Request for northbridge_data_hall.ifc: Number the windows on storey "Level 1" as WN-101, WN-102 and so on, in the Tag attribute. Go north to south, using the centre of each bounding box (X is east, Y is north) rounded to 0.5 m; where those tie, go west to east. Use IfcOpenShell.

First a look at what the model holds.

```python
import ifcopenshell
import ifcopenshell.util.element
import ifcopenshell.util.placement

model = ifcopenshell.open("northbridge_data_hall.ifc")
print(model.schema)
storey = next(s for s in model.by_type("IfcBuildingStorey") if s.Name == "Level 1")
windows = [e for e in ifcopenshell.util.element.get_decomposition(storey) if e.is_a("IfcWindow")]
for e in sorted(windows, key=lambda e: e.id()):
    origin = ifcopenshell.util.placement.get_local_placement(e.ObjectPlacement)[:3, 3]
    print(e.id(), e.Tag, e.Name, origin.round(2) + 0.0, sep=" | ")
```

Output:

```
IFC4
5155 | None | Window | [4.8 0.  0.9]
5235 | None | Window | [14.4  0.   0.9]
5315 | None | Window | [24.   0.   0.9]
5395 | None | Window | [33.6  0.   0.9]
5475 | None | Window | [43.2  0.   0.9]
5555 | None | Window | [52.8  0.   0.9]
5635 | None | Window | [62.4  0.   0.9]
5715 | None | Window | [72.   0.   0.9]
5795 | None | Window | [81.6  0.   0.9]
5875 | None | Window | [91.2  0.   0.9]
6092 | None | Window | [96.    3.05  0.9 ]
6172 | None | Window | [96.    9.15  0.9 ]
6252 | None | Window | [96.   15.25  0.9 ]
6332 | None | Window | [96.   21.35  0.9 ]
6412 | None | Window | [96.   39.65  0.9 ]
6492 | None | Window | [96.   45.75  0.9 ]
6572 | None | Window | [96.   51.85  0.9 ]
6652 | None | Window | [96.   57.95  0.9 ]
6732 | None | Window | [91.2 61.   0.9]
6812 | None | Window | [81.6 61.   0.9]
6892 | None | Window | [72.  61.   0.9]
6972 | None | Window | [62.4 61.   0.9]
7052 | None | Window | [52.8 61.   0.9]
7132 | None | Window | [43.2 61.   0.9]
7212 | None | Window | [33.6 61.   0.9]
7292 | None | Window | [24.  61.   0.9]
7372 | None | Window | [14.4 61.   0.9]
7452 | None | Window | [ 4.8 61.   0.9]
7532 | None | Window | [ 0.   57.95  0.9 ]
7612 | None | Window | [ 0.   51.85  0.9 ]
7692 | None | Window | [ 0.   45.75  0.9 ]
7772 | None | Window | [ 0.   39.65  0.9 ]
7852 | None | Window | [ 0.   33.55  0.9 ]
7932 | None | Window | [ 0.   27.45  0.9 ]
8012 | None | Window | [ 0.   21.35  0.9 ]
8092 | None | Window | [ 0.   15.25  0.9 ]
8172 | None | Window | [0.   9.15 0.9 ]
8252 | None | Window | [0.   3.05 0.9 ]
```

```python
import ifcopenshell
import ifcopenshell.geom
import ifcopenshell.util.element
import ifcopenshell.util.shape

model = ifcopenshell.open("northbridge_data_hall.ifc")
settings = ifcopenshell.geom.settings()
settings.set("use-world-coords", True)


def centre(element):
    shape = ifcopenshell.geom.create_shape(settings, element)
    return ifcopenshell.util.shape.get_bbox_centroid(shape.geometry)


storey = next(s for s in model.by_type("IfcBuildingStorey") if s.Name == "Level 1")
windows = [e for e in ifcopenshell.util.element.get_decomposition(storey) if e.is_a("IfcWindow")]

# Insertion points can sit at a corner or the storey origin, so sort by the geometry (in metres).
centres = {e: centre(e) for e in windows}
windows.sort(key=lambda e: (-round(centres[e][1] / 0.5), centres[e][0]))

for i, e in enumerate(windows, start=1):
    number = f"WN-1{i:02d}"
    e.Tag = number
    print(e.id(), number)

model.write("northbridge_data_hall-out.ifc")
```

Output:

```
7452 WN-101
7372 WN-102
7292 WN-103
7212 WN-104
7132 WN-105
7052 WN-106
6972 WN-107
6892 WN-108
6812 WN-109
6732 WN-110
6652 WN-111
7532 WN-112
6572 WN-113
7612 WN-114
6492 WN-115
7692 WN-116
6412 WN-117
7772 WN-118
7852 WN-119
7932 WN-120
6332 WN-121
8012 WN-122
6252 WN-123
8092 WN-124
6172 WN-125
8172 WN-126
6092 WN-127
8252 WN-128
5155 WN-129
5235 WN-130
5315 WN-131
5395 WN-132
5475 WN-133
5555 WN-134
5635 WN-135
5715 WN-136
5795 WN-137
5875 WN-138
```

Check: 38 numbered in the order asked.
